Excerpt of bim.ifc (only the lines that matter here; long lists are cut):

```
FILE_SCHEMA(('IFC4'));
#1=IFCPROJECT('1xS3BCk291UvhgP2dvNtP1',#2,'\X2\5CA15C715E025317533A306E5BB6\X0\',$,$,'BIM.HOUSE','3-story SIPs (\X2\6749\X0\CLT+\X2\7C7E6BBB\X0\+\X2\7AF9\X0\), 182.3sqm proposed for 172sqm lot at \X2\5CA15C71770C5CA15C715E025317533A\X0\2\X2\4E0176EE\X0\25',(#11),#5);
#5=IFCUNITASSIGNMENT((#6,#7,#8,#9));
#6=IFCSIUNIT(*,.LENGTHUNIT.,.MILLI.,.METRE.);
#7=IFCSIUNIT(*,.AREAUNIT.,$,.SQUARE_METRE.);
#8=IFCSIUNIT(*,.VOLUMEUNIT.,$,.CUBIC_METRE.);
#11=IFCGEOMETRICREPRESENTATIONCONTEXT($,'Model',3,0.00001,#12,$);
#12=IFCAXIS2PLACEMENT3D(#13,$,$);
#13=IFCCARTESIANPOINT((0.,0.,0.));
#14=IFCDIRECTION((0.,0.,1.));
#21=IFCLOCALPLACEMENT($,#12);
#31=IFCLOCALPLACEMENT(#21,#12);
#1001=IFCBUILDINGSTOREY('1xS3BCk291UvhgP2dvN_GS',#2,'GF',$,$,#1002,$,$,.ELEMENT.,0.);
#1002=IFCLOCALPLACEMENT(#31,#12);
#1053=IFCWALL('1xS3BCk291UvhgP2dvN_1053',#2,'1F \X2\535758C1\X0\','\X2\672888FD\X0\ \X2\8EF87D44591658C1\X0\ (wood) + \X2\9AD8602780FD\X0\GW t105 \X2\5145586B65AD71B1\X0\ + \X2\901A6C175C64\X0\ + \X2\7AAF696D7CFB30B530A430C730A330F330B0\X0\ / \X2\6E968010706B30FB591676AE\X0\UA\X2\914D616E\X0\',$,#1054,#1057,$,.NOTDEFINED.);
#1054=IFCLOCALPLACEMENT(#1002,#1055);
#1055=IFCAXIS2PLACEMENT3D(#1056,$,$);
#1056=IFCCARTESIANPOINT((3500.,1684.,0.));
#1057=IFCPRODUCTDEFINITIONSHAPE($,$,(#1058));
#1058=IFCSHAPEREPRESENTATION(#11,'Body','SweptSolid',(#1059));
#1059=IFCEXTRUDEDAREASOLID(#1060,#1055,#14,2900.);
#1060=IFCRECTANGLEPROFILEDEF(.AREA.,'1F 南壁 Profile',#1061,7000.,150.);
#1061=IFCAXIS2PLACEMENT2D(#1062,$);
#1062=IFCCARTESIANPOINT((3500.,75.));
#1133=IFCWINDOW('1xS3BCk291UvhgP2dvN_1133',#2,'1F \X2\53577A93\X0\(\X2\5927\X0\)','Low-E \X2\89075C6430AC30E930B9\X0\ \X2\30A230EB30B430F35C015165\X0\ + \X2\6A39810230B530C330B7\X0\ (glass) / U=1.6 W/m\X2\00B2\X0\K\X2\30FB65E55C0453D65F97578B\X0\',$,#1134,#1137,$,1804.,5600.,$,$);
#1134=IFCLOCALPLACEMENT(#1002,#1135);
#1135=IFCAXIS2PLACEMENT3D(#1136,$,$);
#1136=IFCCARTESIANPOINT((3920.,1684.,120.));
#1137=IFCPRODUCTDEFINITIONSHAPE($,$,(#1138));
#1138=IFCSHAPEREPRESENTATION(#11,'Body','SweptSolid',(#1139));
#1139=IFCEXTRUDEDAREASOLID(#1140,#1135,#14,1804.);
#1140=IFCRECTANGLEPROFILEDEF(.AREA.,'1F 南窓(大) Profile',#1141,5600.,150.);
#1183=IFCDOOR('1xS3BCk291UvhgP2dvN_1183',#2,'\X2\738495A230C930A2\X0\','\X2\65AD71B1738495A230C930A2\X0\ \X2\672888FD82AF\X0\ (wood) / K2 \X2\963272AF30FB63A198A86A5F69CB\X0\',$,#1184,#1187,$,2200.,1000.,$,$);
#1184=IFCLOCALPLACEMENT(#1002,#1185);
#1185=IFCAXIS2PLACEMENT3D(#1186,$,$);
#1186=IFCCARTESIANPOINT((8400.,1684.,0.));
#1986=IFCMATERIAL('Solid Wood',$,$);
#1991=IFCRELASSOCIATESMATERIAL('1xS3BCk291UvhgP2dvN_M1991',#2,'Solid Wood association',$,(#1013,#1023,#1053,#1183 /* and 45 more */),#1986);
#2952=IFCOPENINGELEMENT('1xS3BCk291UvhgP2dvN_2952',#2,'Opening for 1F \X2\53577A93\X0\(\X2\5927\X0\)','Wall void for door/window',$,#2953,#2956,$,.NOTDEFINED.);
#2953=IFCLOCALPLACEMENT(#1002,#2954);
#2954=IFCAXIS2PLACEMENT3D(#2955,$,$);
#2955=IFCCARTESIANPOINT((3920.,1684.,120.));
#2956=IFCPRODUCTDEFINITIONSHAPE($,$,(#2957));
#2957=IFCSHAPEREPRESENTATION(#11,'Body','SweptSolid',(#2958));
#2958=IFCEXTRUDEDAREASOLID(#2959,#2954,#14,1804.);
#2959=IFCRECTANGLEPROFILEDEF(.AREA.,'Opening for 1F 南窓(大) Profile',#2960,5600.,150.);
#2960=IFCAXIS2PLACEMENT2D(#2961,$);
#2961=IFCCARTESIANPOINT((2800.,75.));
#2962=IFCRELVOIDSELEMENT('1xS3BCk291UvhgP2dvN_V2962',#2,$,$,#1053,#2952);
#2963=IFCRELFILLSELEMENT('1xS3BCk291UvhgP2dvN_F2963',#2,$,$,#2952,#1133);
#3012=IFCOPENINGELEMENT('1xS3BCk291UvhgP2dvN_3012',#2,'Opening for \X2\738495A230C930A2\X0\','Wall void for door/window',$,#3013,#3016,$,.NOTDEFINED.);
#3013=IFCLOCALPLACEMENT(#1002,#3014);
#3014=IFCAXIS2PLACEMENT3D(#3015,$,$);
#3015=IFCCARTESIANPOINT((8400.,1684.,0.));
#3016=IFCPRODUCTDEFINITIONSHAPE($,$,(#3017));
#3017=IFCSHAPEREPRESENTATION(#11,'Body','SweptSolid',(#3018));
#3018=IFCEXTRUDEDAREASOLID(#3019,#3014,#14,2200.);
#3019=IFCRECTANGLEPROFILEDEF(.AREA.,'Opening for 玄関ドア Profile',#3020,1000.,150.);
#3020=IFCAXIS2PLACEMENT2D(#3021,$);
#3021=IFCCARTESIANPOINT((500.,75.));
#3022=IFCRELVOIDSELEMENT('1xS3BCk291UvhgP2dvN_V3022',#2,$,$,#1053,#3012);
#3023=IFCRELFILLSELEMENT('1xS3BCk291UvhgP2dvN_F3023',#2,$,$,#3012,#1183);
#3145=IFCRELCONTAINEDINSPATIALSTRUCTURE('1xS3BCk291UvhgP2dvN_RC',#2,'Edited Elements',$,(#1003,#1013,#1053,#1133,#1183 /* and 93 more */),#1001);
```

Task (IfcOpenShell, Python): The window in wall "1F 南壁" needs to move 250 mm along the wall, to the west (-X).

```python
import ifcopenshell
import ifcopenshell.api.geometry
import ifcopenshell.util.placement
import ifcopenshell.util.unit

model = ifcopenshell.open("bim.ifc")
unit_scale = ifcopenshell.util.unit.calculate_unit_scale(model)

window = model.by_id(1133)
opening = window.FillsVoids[0].RelatingOpeningElement
wall = opening.VoidsElements[0].RelatingBuildingElement

wall_matrix = ifcopenshell.util.placement.get_local_placement(wall.ObjectPlacement)
shift = wall_matrix[:3, 0] * -0.25 / unit_scale
before = ifcopenshell.util.placement.get_local_placement(window.ObjectPlacement)[:3, 3].copy()

# The window is not placed relative to its opening, so move both.
for product in (opening, window):
    matrix = ifcopenshell.util.placement.get_local_placement(product.ObjectPlacement)
    matrix[:3, 3] += shift
    ifcopenshell.api.geometry.edit_object_placement(model, product=product, matrix=matrix, is_si=False)

after = ifcopenshell.util.placement.get_local_placement(window.ObjectPlacement)[:3, 3]
print("window moved by", (after - before).round(3) + 0.0)

model.write("bim_edited.ifc")
```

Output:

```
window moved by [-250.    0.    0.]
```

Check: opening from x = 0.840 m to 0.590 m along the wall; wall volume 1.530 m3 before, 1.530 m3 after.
